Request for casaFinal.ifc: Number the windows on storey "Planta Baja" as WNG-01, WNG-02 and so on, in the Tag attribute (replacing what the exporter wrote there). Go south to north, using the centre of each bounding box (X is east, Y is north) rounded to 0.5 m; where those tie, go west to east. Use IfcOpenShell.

First a look at what the model holds.

```python
import ifcopenshell
import ifcopenshell.util.element
import ifcopenshell.util.placement

model = ifcopenshell.open("casaFinal.ifc")
print(model.schema)
storey = next(s for s in model.by_type("IfcBuildingStorey") if s.Name == "Planta Baja")
windows = [e for e in ifcopenshell.util.element.get_decomposition(storey) if e.is_a("IfcWindow")]
for e in sorted(windows, key=lambda e: e.id()):
    origin = ifcopenshell.util.placement.get_local_placement(e.ObjectPlacement)[:3, 3]
    print(e.id(), e.Tag, e.Name, origin.round(2) + 0.0, sep=" | ")
```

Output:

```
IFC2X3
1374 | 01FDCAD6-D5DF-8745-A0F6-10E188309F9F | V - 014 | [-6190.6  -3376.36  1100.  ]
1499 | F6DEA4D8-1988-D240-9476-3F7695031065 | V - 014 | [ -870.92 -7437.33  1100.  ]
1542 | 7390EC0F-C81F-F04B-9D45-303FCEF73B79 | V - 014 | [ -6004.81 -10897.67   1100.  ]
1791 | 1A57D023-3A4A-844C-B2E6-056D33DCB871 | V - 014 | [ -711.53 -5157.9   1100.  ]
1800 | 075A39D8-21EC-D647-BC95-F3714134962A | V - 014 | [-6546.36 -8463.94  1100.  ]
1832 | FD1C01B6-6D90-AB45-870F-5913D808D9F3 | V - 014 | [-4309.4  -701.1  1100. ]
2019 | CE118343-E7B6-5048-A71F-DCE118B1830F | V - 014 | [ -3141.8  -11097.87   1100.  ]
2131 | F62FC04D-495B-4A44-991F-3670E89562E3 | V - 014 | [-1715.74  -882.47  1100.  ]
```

```python
import ifcopenshell
import ifcopenshell.geom
import ifcopenshell.util.element
import ifcopenshell.util.shape

model = ifcopenshell.open("casaFinal.ifc")
settings = ifcopenshell.geom.settings()
settings.set("use-world-coords", True)


def centre(element):
    shape = ifcopenshell.geom.create_shape(settings, element)
    return ifcopenshell.util.shape.get_bbox_centroid(shape.geometry)


storey = next(s for s in model.by_type("IfcBuildingStorey") if s.Name == "Planta Baja")
windows = [e for e in ifcopenshell.util.element.get_decomposition(storey) if e.is_a("IfcWindow")]

# Insertion points can sit at a corner or the storey origin, so sort by the geometry (in metres).
centres = {e: centre(e) for e in windows}
windows.sort(key=lambda e: (round(centres[e][1] / 0.5), centres[e][0]))

for i, e in enumerate(windows, start=1):
    number = f"WNG-{i:02d}"
    e.Tag = number
    print(e.id(), number)

model.write("casaFinal_rev.ifc")
```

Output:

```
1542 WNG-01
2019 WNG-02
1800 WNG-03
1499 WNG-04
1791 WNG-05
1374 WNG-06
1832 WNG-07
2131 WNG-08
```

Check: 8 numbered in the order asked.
